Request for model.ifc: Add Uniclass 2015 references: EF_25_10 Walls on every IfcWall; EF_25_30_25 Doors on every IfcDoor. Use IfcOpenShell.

First a look at what the model holds.

```python
import ifcopenshell

model = ifcopenshell.open("model.ifc")
print(model.schema)
print("classifications:", [c.Name for c in model.by_type("IfcClassification")])
for ifc_class in ("IfcDoor", "IfcRoof", "IfcStair", "IfcWall", "IfcWindow"):
    print(ifc_class, len(model.by_type(ifc_class)))
```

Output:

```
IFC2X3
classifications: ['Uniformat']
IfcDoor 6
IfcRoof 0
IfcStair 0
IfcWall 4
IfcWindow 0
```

```python
import ifcopenshell
import ifcopenshell.api.classification

model = ifcopenshell.open("model.ifc")

# IFC2X3 requires Source and Edition and has no link from the project to the system.
system = model.create_entity("IfcClassification", Source="NBS", Edition="2015", Name="Uniclass 2015")

codes = {
    "IfcWall": ("EF_25_10", "Walls"),
    "IfcDoor": ("EF_25_30_25", "Doors"),
}
for ifc_class, (code, name) in codes.items():
    products = model.by_type(ifc_class)
    ifcopenshell.api.classification.add_reference(
        model, products=products, classification=system, identification=code, name=name
    )
    print(code, len(products))

model.write("model_updated.ifc")
```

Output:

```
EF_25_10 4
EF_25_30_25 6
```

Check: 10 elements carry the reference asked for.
